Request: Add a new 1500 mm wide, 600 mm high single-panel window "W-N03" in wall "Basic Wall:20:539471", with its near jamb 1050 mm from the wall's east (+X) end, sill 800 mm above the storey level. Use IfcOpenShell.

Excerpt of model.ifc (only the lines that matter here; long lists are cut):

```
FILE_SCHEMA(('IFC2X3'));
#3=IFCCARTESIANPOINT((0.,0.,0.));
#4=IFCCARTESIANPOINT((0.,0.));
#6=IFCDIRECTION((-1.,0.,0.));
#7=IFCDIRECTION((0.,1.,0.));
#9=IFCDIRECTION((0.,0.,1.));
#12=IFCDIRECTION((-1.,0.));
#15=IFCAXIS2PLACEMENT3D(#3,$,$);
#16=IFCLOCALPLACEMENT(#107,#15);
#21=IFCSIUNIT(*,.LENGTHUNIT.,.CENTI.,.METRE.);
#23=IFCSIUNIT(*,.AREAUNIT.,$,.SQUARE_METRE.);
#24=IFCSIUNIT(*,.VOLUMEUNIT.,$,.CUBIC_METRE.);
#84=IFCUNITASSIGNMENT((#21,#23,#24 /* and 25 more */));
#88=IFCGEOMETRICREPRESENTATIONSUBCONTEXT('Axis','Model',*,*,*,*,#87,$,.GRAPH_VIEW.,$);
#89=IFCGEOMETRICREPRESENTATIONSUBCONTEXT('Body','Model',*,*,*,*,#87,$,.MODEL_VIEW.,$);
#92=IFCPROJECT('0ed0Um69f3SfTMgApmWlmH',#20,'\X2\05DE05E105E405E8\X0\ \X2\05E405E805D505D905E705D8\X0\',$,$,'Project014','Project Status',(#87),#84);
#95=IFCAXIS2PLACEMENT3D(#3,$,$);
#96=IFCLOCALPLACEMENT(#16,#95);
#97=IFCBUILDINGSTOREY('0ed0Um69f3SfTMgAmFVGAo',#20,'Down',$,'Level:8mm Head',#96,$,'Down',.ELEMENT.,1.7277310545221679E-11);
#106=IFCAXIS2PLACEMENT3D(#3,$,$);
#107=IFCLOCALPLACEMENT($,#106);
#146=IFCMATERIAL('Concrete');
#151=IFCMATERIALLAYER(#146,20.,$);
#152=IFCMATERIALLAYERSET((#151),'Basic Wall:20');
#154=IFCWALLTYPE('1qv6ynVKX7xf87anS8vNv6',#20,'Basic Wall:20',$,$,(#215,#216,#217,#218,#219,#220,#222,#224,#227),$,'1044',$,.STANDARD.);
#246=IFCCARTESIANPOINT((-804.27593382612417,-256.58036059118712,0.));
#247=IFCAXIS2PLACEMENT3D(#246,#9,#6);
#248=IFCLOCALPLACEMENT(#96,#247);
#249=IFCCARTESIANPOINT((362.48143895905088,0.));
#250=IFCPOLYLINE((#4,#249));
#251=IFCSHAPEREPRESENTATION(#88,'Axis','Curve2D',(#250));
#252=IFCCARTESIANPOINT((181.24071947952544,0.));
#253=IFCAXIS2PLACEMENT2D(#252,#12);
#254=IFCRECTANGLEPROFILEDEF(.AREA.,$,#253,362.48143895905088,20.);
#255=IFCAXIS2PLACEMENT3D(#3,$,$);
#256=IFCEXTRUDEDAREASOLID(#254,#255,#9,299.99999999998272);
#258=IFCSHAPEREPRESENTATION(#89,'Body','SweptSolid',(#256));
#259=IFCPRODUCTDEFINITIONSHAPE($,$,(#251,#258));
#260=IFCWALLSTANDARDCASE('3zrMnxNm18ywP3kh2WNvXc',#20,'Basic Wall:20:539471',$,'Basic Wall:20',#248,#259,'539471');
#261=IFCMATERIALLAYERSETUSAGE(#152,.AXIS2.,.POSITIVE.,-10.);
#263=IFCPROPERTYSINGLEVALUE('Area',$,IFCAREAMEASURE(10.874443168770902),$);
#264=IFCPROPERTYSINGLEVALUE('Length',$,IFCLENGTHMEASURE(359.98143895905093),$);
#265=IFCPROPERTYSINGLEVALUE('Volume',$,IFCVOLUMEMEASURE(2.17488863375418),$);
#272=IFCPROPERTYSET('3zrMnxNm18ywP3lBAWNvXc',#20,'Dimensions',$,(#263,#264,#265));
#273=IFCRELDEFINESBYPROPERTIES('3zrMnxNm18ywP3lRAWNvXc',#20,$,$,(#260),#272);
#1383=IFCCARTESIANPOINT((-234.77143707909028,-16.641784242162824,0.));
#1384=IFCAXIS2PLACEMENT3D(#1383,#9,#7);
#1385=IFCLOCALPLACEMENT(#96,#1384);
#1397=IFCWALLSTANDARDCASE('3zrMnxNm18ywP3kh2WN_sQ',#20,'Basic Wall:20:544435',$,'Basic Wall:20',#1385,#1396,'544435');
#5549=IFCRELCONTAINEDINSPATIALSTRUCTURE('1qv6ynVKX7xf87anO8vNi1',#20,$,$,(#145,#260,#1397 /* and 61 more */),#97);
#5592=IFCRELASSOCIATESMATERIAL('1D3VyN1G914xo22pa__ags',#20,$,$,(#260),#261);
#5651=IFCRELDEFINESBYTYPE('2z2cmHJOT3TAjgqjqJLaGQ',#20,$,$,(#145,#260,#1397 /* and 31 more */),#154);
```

```python
import numpy as np
import ifcopenshell
import ifcopenshell.api.feature
import ifcopenshell.api.geometry
import ifcopenshell.api.pset
import ifcopenshell.api.root
import ifcopenshell.api.spatial
import ifcopenshell.api.type
import ifcopenshell.geom
import ifcopenshell.util.element
import ifcopenshell.util.placement
import ifcopenshell.util.representation
import ifcopenshell.util.shape
import ifcopenshell.util.unit

model = ifcopenshell.open("model.ifc")
unit_scale = ifcopenshell.util.unit.calculate_unit_scale(model)
area_scale = ifcopenshell.util.unit.calculate_unit_scale(model, "AREAUNIT")
volume_scale = ifcopenshell.util.unit.calculate_unit_scale(model, "VOLUMEUNIT")
settings = ifcopenshell.geom.settings()


def volume(element):
    """Net volume in cubic metres, openings subtracted."""
    shape = ifcopenshell.geom.create_shape(settings, element)
    return ifcopenshell.util.shape.get_volume(shape.geometry)


wall = model.by_guid("3zrMnxNm18ywP3kh2WNvXc")
storey = ifcopenshell.util.element.get_container(wall, ifc_class="IfcBuildingStorey")
context = ifcopenshell.util.representation.get_context(model, "Model", "Body", "MODEL_VIEW")
before = volume(wall)

width, height, from_end, sill = 1.5, 0.6, 1.05, 0.8  # metres

# The wall runs along its own X axis, and the end named is its -X end.
wall_shape = ifcopenshell.geom.create_shape(settings, wall)
x, y, z = ifcopenshell.util.shape.get_vertices(wall_shape.geometry).T
start = x.min() + from_end
face, thickness = float(y.min()), float(y.max() - y.min())
wall_matrix = ifcopenshell.util.placement.get_local_placement(wall.ObjectPlacement)
level = ifcopenshell.util.placement.get_local_placement(storey.ObjectPlacement)[2, 3]


def in_wall(x, y):
    """Placement at x, y metres in the wall's axes, at sill height."""
    matrix = wall_matrix.copy()
    matrix[:, 3] = wall_matrix @ np.array([x / unit_scale, y / unit_scale, 0.0, 1.0])
    matrix[2, 3] = level + sill / unit_scale
    return matrix


# Opening: a box that overshoots both wall faces by 50 mm.
opening = ifcopenshell.api.root.create_entity(model, ifc_class="IfcOpeningElement")
box = ifcopenshell.api.geometry.add_wall_representation(
    model, context=context, length=width, height=height, thickness=thickness + 0.1
)
ifcopenshell.api.geometry.assign_representation(model, product=opening, representation=box)
ifcopenshell.api.geometry.edit_object_placement(model, product=opening, matrix=in_wall(start, face - 0.05), is_si=False)
ifcopenshell.api.feature.add_feature(model, feature=opening, element=wall)

window = ifcopenshell.api.root.create_entity(model, ifc_class="IfcWindow", name="W-N03")
window.OverallWidth, window.OverallHeight = width / unit_scale, height / unit_scale
body = ifcopenshell.api.geometry.add_window_representation(
    model,
    context=context,
    overall_width=window.OverallWidth,
    overall_height=window.OverallHeight,
    partition_type="SINGLE_PANEL",
)
ifcopenshell.api.geometry.assign_representation(model, product=window, representation=body)
ifcopenshell.api.spatial.assign_container(model, products=[window], relating_structure=storey)
fills = ifcopenshell.api.feature.add_filling(model, opening=opening, element=window)
fills.OwnerHistory = window.OwnerHistory  # required in IFC2X3

# IFC2X3 keeps the operation on the window style.
style = ifcopenshell.api.root.create_entity(model, ifc_class="IfcWindowStyle", name="W-N03")
style.OperationType, style.ConstructionType = "SINGLE_PANEL", "NOTDEFINED"
style.ParameterTakesPrecedence = style.Sizeable = False
ifcopenshell.api.type.assign_type(model, related_objects=[window], relating_type=style)

# Centre the window in the wall's thickness.
ifcopenshell.api.geometry.edit_object_placement(model, product=window, matrix=in_wall(start, face), is_si=False)
window_shape = ifcopenshell.geom.create_shape(settings, window)
depth = ifcopenshell.util.shape.get_vertices(window_shape.geometry)[:, 1]
offset = face + thickness / 2 - (depth.min() + depth.max()) / 2
ifcopenshell.api.geometry.edit_object_placement(model, product=window, matrix=in_wall(start, offset), is_si=False)

after = volume(wall)

# Update the wall's stored quantities.
pset = model.by_id(ifcopenshell.util.element.get_pset(wall, "Dimensions", should_inherit=False)["id"])
ifcopenshell.api.pset.edit_pset(model, pset=pset, properties={
    "Area": model.create_entity("IfcAreaMeasure", after / thickness / area_scale),
    "Volume": model.create_entity("IfcVolumeMeasure", after / volume_scale),
})

print(f"wall volume {before:.3f} -> {after:.3f} m3")

model.write("model_edited.ifc")
```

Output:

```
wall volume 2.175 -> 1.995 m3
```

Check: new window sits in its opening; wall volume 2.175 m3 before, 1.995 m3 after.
